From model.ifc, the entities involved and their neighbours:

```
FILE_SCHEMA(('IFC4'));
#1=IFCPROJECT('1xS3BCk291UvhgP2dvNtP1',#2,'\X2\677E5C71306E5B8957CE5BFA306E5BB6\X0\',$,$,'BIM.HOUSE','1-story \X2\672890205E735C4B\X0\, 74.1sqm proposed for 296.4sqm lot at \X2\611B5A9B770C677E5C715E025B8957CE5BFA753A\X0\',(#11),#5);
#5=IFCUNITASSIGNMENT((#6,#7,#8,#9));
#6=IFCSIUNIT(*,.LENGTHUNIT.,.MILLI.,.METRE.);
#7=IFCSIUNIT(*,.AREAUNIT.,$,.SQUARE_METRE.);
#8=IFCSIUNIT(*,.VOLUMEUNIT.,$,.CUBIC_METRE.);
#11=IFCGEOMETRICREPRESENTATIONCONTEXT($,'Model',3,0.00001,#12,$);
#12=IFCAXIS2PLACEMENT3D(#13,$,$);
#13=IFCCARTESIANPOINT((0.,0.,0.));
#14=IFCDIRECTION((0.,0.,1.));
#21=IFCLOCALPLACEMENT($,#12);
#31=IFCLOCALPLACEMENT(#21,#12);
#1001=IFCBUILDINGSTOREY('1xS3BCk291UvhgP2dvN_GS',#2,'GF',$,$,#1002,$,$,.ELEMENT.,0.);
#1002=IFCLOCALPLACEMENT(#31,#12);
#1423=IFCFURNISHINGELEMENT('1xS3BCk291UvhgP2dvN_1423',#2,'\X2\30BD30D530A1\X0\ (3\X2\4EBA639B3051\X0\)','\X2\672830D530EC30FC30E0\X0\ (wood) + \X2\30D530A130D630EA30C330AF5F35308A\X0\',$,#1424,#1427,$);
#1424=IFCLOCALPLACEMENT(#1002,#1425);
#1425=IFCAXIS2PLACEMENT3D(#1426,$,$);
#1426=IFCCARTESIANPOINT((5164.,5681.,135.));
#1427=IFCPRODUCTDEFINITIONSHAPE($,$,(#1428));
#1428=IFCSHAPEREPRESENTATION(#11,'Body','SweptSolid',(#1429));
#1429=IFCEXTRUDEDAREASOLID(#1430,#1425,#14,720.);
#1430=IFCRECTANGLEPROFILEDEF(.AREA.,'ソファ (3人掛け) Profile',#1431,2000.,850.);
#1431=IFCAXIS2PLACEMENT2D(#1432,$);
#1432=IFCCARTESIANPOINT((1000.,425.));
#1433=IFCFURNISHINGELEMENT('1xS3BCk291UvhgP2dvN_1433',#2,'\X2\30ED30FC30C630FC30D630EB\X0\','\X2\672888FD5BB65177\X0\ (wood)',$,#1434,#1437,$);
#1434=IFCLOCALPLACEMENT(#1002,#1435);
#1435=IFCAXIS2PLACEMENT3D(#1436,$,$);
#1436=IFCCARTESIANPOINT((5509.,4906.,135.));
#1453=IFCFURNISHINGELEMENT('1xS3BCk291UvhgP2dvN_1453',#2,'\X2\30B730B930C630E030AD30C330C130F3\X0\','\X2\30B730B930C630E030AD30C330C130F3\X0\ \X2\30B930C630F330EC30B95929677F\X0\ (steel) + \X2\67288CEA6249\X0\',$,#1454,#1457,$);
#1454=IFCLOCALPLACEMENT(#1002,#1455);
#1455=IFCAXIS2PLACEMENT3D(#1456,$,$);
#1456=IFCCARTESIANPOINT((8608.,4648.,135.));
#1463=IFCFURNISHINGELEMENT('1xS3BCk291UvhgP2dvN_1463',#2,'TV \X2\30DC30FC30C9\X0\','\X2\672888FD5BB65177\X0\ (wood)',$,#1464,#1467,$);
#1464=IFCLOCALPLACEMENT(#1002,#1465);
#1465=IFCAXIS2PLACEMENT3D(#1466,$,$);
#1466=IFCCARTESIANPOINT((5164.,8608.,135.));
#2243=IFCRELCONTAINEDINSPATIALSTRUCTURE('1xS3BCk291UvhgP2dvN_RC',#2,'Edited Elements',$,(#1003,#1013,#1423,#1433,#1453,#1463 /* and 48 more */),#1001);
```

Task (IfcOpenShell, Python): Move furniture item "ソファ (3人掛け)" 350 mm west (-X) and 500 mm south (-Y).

```python
import ifcopenshell
import ifcopenshell.api.geometry
import ifcopenshell.util.placement
import ifcopenshell.util.unit

model = ifcopenshell.open("model.ifc")
unit_scale = ifcopenshell.util.unit.calculate_unit_scale(model)

item = model.by_guid("1xS3BCk291UvhgP2dvN_1423")
matrix = ifcopenshell.util.placement.get_local_placement(item.ObjectPlacement)
matrix[0, 3] -= 0.35 / unit_scale
matrix[1, 3] -= 0.5 / unit_scale
ifcopenshell.api.geometry.edit_object_placement(model, product=item, matrix=matrix, is_si=False)

print(ifcopenshell.util.placement.get_local_placement(item.ObjectPlacement).round(3) + 0.0)

model.write("model_updated.ifc")
```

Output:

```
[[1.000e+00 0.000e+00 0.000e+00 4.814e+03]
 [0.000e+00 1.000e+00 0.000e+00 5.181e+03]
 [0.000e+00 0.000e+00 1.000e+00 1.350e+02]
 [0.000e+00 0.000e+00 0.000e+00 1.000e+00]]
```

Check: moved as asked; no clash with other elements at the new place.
